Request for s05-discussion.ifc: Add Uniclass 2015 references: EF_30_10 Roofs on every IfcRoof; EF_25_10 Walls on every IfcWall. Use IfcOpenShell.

First a look at what the model holds.

```python
import ifcopenshell

model = ifcopenshell.open("s05-discussion.ifc")
print(model.schema)
print("classifications:", [c.Name for c in model.by_type("IfcClassification")])
for ifc_class in ("IfcDoor", "IfcRoof", "IfcStair", "IfcWall", "IfcWindow"):
    print(ifc_class, len(model.by_type(ifc_class)))
```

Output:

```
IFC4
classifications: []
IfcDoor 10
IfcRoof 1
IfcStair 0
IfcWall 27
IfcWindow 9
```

```python
import ifcopenshell
import ifcopenshell.api.classification

model = ifcopenshell.open("s05-discussion.ifc")

system = ifcopenshell.api.classification.add_classification(model, classification="Uniclass 2015")

codes = {
    "IfcRoof": ("EF_30_10", "Roofs"),
    "IfcWall": ("EF_25_10", "Walls"),
}
for ifc_class, (code, name) in codes.items():
    products = model.by_type(ifc_class)
    ifcopenshell.api.classification.add_reference(
        model, products=products, classification=system, identification=code, name=name
    )
    print(code, len(products))

model.write("s05-discussion_rev.ifc")
```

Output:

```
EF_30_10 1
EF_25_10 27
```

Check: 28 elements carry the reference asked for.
